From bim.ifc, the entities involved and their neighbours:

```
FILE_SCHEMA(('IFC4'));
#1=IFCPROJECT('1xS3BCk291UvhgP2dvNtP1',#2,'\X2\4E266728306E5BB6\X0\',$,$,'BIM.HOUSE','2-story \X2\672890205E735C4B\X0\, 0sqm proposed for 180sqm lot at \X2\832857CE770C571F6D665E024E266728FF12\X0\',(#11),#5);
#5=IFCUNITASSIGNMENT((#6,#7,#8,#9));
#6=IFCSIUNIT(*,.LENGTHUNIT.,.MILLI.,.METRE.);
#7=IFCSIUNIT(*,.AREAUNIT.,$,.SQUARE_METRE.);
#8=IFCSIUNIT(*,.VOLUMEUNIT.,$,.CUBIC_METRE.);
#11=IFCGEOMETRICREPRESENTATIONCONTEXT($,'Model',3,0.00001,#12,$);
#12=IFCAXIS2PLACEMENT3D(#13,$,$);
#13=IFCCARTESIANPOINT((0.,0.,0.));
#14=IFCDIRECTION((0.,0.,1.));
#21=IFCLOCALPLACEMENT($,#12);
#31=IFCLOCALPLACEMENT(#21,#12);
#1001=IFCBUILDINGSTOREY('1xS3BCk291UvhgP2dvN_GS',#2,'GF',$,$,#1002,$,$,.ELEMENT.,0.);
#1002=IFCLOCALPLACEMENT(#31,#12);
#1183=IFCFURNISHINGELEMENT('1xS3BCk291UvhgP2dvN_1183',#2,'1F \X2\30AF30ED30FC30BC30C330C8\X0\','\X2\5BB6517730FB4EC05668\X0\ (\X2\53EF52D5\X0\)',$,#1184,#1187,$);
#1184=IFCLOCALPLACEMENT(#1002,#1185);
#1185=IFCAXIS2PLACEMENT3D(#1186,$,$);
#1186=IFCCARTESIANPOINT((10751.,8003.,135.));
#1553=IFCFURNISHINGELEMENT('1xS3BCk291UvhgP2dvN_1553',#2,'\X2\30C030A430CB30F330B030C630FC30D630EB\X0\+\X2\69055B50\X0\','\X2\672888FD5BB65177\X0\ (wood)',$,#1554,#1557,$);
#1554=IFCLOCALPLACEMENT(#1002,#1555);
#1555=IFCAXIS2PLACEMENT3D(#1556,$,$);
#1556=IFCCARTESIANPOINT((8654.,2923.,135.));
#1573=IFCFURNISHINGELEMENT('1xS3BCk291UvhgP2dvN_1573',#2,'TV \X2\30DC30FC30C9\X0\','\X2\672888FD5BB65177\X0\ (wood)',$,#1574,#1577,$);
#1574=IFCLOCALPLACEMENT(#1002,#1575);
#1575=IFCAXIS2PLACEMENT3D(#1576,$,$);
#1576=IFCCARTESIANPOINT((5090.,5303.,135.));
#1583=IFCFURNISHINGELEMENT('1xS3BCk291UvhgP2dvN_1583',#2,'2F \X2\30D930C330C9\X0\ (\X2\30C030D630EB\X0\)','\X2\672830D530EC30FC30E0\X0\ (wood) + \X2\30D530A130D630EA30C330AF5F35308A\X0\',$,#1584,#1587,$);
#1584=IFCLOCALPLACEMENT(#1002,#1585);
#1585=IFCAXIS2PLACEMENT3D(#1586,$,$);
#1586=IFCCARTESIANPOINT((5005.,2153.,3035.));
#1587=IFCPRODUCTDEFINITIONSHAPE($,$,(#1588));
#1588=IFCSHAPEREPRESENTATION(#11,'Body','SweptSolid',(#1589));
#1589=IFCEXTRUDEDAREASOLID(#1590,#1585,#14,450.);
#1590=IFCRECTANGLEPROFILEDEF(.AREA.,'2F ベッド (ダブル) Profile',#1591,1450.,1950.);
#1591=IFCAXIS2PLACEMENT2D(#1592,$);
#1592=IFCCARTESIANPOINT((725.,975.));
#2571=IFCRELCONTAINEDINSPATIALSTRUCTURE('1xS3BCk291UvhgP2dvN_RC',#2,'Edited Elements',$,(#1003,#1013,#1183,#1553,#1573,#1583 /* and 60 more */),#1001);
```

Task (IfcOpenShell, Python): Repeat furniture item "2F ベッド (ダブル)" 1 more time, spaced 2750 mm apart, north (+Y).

```python
import numpy as np
import ifcopenshell
import ifcopenshell.api.geometry
import ifcopenshell.api.root
import ifcopenshell.util.element
import ifcopenshell.util.placement

model = ifcopenshell.open("bim.ifc")


def reuse_history(source, copy):
    """copy_class also copies each property set's owner history, people and application; keep the originals."""
    for rel in copy.IsDefinedBy:
        if rel.is_a("IfcRelDefinesByProperties") and (history := rel.RelatingPropertyDefinition.OwnerHistory):
            rel.RelatingPropertyDefinition.OwnerHistory = source.OwnerHistory
            ifcopenshell.util.element.remove_deep2(model, history)


source = model.by_guid("1xS3BCk291UvhgP2dvN_1583")
base = ifcopenshell.util.placement.get_local_placement(source.ObjectPlacement)
step = np.array([0.0, 1.0, 0.0]) * 2750.0

for i in range(1, 2):
    copy = ifcopenshell.api.root.copy_class(model, product=source)
    copy.Representation = ifcopenshell.util.element.copy_deep(
        model, source.Representation, exclude=["IfcGeometricRepresentationContext", "IfcRepresentationMap"]
    )
    reuse_history(source, copy)
    matrix = base.copy()
    matrix[:3, 3] += i * step
    print("added at", matrix[:3, 3].round(3) + 0.0)
    ifcopenshell.api.geometry.edit_object_placement(model, product=copy, matrix=matrix, is_si=False)

model.write("bim_rev.ifc")
```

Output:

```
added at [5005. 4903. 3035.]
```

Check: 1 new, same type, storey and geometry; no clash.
